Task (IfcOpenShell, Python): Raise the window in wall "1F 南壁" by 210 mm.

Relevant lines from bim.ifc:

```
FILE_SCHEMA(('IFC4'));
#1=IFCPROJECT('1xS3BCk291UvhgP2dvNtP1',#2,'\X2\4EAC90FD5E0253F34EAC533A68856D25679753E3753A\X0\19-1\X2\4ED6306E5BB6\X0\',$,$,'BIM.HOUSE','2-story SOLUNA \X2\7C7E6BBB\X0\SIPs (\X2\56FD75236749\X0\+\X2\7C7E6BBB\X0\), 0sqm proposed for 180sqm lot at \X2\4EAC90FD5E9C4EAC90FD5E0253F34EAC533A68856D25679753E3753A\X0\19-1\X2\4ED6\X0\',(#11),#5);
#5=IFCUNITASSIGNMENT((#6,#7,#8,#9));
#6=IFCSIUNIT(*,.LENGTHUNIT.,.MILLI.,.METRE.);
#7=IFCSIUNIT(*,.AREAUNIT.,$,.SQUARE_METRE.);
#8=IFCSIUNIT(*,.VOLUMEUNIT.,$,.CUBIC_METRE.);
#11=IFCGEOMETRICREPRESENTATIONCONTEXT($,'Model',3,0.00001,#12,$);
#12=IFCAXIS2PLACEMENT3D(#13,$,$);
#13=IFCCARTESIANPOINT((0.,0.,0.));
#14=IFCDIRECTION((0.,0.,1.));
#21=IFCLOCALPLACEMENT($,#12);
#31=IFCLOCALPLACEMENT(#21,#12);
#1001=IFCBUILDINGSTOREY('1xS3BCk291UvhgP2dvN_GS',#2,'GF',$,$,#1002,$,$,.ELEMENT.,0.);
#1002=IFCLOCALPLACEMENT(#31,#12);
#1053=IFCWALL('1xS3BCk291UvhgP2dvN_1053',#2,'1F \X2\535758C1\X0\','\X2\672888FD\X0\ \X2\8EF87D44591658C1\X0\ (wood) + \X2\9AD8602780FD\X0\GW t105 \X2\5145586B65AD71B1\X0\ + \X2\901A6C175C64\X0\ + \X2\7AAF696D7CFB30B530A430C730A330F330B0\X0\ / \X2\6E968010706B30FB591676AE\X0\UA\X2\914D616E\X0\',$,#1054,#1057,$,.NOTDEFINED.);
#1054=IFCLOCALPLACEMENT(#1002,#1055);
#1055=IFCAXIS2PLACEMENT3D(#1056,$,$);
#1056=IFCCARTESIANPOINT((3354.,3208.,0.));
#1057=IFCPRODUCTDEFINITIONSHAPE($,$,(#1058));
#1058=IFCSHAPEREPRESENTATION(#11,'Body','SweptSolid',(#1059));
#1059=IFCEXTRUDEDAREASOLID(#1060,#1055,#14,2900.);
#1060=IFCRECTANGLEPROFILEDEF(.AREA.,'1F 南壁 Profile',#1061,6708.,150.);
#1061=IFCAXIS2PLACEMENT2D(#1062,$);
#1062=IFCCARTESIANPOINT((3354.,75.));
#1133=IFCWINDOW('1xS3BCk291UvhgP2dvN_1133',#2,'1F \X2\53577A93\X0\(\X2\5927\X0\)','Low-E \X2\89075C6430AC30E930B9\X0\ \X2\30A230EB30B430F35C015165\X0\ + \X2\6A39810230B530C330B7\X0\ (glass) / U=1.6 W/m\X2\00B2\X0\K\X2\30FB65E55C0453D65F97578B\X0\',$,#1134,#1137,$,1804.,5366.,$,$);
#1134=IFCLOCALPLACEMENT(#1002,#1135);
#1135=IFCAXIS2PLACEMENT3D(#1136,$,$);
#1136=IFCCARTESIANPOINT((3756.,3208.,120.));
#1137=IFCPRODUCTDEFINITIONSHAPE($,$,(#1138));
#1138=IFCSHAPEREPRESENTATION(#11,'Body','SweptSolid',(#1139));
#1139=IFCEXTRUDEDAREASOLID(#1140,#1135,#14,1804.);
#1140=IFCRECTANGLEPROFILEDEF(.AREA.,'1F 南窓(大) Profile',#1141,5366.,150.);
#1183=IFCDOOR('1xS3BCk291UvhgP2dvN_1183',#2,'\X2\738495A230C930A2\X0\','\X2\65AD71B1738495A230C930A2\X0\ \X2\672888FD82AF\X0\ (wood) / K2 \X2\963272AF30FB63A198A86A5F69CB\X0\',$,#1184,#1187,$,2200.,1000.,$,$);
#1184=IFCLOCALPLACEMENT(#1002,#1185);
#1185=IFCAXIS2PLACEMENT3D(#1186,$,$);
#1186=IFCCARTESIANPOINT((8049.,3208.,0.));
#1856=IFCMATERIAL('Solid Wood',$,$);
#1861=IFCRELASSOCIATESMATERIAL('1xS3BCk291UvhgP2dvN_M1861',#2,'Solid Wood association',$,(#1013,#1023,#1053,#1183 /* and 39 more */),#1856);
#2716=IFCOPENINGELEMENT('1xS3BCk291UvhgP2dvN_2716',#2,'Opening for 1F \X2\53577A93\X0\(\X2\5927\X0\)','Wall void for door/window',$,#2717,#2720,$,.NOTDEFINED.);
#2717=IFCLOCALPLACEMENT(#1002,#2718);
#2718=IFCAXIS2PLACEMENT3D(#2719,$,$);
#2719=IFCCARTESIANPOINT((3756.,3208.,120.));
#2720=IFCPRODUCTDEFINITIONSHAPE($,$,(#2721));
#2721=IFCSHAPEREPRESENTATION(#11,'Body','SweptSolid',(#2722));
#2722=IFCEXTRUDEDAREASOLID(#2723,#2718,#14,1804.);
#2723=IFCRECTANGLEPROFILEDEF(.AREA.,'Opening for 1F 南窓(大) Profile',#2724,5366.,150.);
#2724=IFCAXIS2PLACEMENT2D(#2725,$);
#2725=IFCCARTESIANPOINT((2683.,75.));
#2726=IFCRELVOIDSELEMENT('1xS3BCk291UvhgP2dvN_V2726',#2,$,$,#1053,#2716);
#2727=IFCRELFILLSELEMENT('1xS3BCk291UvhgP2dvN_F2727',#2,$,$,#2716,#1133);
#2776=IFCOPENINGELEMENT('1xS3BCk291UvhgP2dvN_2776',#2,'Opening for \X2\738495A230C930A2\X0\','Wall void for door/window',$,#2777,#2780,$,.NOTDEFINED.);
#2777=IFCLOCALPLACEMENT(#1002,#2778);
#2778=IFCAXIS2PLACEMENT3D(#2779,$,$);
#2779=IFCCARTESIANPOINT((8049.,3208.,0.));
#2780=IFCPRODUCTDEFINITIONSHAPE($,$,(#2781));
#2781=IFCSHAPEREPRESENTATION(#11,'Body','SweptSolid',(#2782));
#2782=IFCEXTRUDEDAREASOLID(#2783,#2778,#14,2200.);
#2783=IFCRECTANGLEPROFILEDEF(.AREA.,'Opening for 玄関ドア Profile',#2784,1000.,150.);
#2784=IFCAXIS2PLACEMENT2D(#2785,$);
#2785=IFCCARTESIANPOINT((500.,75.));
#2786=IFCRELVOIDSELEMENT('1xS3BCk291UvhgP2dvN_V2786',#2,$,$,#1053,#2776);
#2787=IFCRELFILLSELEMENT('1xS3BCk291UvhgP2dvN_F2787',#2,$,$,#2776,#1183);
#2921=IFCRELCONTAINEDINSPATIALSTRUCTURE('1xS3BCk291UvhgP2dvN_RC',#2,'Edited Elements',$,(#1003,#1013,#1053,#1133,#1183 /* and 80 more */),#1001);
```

```python
import numpy as np
import ifcopenshell
import ifcopenshell.api.geometry
import ifcopenshell.util.placement
import ifcopenshell.util.unit

model = ifcopenshell.open("bim.ifc")
unit_scale = ifcopenshell.util.unit.calculate_unit_scale(model)

window = model.by_guid("1xS3BCk291UvhgP2dvN_1133")
opening = window.FillsVoids[0].RelatingOpeningElement
dz = 0.21 / unit_scale

shift = np.array([0.0, 0.0, dz])
# The window is not placed relative to its opening, so move both.
for product in (opening, window):
    matrix = ifcopenshell.util.placement.get_local_placement(product.ObjectPlacement)
    matrix[:3, 3] += shift
    ifcopenshell.api.geometry.edit_object_placement(model, product=product, matrix=matrix, is_si=False)

print(f"moved by {dz * unit_scale:+.3f} m")

model.write("bim-out.ifc")
```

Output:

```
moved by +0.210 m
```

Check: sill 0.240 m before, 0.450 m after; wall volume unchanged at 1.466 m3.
